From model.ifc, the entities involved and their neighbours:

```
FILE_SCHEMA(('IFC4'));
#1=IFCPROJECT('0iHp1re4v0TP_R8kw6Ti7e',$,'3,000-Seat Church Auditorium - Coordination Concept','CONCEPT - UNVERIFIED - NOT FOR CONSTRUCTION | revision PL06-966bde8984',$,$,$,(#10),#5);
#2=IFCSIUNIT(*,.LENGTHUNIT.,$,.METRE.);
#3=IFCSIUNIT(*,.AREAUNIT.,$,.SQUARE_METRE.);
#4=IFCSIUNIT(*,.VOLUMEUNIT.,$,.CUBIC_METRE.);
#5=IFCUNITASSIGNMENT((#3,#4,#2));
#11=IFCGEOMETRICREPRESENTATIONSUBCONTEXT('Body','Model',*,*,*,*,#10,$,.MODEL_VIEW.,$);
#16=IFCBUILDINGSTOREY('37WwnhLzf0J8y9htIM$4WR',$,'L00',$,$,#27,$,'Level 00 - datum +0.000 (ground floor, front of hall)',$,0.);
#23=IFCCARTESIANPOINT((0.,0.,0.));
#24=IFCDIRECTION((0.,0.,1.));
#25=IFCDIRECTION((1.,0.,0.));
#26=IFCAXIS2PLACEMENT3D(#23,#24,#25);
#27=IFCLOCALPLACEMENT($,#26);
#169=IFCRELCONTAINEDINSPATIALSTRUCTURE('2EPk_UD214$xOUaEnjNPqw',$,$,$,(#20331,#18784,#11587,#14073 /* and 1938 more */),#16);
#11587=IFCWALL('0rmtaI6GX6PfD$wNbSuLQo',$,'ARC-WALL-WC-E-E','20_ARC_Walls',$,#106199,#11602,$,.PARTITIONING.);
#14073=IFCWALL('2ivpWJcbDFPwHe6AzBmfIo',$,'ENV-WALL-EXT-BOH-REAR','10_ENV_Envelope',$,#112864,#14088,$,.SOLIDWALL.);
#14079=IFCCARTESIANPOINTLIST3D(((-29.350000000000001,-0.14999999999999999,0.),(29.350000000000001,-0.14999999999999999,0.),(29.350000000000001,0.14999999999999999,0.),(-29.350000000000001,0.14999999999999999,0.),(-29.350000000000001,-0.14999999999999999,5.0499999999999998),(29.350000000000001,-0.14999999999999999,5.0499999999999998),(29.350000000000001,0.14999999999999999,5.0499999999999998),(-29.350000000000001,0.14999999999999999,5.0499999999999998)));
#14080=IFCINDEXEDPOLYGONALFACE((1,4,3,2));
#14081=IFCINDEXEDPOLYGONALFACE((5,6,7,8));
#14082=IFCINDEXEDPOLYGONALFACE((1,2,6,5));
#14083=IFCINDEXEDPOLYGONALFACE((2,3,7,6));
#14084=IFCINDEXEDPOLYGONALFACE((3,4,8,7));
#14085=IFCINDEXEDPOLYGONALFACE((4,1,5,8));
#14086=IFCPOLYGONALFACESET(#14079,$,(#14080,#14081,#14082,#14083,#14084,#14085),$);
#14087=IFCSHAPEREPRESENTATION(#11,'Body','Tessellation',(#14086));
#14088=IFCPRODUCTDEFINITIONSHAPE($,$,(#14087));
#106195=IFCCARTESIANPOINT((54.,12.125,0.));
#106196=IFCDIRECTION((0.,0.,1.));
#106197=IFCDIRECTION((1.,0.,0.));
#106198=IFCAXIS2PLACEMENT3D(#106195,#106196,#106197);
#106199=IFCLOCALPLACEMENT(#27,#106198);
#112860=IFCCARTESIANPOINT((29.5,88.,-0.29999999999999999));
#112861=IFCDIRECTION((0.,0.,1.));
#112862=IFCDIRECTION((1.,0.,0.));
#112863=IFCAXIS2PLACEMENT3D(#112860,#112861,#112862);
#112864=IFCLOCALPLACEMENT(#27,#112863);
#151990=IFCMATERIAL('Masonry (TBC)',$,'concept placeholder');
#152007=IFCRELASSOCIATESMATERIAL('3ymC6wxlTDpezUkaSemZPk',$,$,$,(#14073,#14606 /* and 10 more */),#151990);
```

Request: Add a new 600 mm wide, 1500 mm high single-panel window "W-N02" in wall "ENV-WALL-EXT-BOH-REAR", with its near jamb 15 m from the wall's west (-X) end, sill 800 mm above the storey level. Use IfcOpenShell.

```python
import numpy as np
import ifcopenshell
import ifcopenshell.api.feature
import ifcopenshell.api.geometry
import ifcopenshell.api.root
import ifcopenshell.api.spatial
import ifcopenshell.geom
import ifcopenshell.util.element
import ifcopenshell.util.placement
import ifcopenshell.util.representation
import ifcopenshell.util.shape
import ifcopenshell.util.unit

model = ifcopenshell.open("model.ifc")
unit_scale = ifcopenshell.util.unit.calculate_unit_scale(model)
settings = ifcopenshell.geom.settings()


def volume(element):
    """Net volume in cubic metres, openings subtracted."""
    shape = ifcopenshell.geom.create_shape(settings, element)
    return ifcopenshell.util.shape.get_volume(shape.geometry)


wall = model.by_guid("2ivpWJcbDFPwHe6AzBmfIo")
storey = ifcopenshell.util.element.get_container(wall, ifc_class="IfcBuildingStorey")
context = ifcopenshell.util.representation.get_context(model, "Model", "Body", "MODEL_VIEW")
before = volume(wall)

width, height, from_end, sill = 0.6, 1.5, 15, 0.8  # metres

# The wall runs along its own X axis, and the end named is its -X end.
wall_shape = ifcopenshell.geom.create_shape(settings, wall)
x, y, z = ifcopenshell.util.shape.get_vertices(wall_shape.geometry).T
start = x.min() + from_end
face, thickness = float(y.min()), float(y.max() - y.min())
wall_matrix = ifcopenshell.util.placement.get_local_placement(wall.ObjectPlacement)
level = ifcopenshell.util.placement.get_local_placement(storey.ObjectPlacement)[2, 3]


def in_wall(x, y):
    """Placement at x, y metres in the wall's axes, at sill height."""
    matrix = wall_matrix.copy()
    matrix[:, 3] = wall_matrix @ np.array([x / unit_scale, y / unit_scale, 0.0, 1.0])
    matrix[2, 3] = level + sill / unit_scale
    return matrix


# Opening: a box that overshoots both wall faces by 50 mm.
opening = ifcopenshell.api.root.create_entity(model, ifc_class="IfcOpeningElement", predefined_type="OPENING")
box = ifcopenshell.api.geometry.add_wall_representation(
    model, context=context, length=width, height=height, thickness=thickness + 0.1
)
ifcopenshell.api.geometry.assign_representation(model, product=opening, representation=box)
ifcopenshell.api.geometry.edit_object_placement(model, product=opening, matrix=in_wall(start, face - 0.05), is_si=False)
ifcopenshell.api.feature.add_feature(model, feature=opening, element=wall)

window = ifcopenshell.api.root.create_entity(model, ifc_class="IfcWindow", name="W-N02", predefined_type="WINDOW")
window.OverallWidth, window.OverallHeight = width / unit_scale, height / unit_scale
window.PartitioningType = "SINGLE_PANEL"
body = ifcopenshell.api.geometry.add_window_representation(
    model,
    context=context,
    overall_width=window.OverallWidth,
    overall_height=window.OverallHeight,
    partition_type="SINGLE_PANEL",
)
ifcopenshell.api.geometry.assign_representation(model, product=window, representation=body)
ifcopenshell.api.spatial.assign_container(model, products=[window], relating_structure=storey)
ifcopenshell.api.feature.add_filling(model, opening=opening, element=window)

# Centre the window in the wall's thickness.
ifcopenshell.api.geometry.edit_object_placement(model, product=window, matrix=in_wall(start, face), is_si=False)
window_shape = ifcopenshell.geom.create_shape(settings, window)
depth = ifcopenshell.util.shape.get_vertices(window_shape.geometry)[:, 1]
offset = face + thickness / 2 - (depth.min() + depth.max()) / 2
ifcopenshell.api.geometry.edit_object_placement(model, product=window, matrix=in_wall(start, offset), is_si=False)

after = volume(wall)

print(f"wall volume {before:.3f} -> {after:.3f} m3")

model.write("model_edited.ifc")
```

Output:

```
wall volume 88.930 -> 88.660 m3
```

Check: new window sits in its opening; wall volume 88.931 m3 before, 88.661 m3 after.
